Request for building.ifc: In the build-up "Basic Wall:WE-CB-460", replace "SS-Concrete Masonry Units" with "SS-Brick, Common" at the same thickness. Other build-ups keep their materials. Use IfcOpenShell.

First a look at what the model holds.

```python
import ifcopenshell
import ifcopenshell.util.element

model = ifcopenshell.open("building.ifc")
print(model.schema)
for layer_set in model.by_type("IfcMaterialLayerSet"):
    if layer_set.LayerSetName == "Basic Wall:WE-CB-460":
        for layer in layer_set.MaterialLayers:
            print(layer.id(), layer.Material and layer.Material.Name, layer.LayerThickness, sep=" | ")
        print(len(ifcopenshell.util.element.get_elements_by_material(model, layer_set)), "elements and types use it")
print(sorted(m.Name for m in model.by_type("IfcMaterial") if m.Name)[:60])
```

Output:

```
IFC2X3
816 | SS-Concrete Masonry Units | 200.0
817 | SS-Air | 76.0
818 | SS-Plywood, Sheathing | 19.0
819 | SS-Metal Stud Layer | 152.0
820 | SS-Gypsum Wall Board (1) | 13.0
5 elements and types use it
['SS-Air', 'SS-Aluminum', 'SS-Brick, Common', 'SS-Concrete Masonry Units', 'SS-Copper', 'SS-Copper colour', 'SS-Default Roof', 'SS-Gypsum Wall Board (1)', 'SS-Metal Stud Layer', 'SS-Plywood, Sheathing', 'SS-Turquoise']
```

```python
import ifcopenshell
import ifcopenshell.api.material

model = ifcopenshell.open("building.ifc")

layer_set = next(s for s in model.by_type("IfcMaterialLayerSet") if s.LayerSetName == "Basic Wall:WE-CB-460")
layer = next(l for l in layer_set.MaterialLayers if l.Material and l.Material.Name == "SS-Concrete Masonry Units")
material = next(m for m in model.by_type("IfcMaterial") if m.Name == "SS-Brick, Common")

# Point this one layer at the other material; renaming the old one would change it everywhere.
ifcopenshell.api.material.edit_layer(model, layer=layer, attributes={}, material=material)

print([l.Material.Name if l.Material else None for l in layer_set.MaterialLayers])

model.write("building-out.ifc")
```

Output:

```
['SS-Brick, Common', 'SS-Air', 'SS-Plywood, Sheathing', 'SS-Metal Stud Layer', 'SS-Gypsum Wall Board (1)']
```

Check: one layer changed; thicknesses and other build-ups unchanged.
